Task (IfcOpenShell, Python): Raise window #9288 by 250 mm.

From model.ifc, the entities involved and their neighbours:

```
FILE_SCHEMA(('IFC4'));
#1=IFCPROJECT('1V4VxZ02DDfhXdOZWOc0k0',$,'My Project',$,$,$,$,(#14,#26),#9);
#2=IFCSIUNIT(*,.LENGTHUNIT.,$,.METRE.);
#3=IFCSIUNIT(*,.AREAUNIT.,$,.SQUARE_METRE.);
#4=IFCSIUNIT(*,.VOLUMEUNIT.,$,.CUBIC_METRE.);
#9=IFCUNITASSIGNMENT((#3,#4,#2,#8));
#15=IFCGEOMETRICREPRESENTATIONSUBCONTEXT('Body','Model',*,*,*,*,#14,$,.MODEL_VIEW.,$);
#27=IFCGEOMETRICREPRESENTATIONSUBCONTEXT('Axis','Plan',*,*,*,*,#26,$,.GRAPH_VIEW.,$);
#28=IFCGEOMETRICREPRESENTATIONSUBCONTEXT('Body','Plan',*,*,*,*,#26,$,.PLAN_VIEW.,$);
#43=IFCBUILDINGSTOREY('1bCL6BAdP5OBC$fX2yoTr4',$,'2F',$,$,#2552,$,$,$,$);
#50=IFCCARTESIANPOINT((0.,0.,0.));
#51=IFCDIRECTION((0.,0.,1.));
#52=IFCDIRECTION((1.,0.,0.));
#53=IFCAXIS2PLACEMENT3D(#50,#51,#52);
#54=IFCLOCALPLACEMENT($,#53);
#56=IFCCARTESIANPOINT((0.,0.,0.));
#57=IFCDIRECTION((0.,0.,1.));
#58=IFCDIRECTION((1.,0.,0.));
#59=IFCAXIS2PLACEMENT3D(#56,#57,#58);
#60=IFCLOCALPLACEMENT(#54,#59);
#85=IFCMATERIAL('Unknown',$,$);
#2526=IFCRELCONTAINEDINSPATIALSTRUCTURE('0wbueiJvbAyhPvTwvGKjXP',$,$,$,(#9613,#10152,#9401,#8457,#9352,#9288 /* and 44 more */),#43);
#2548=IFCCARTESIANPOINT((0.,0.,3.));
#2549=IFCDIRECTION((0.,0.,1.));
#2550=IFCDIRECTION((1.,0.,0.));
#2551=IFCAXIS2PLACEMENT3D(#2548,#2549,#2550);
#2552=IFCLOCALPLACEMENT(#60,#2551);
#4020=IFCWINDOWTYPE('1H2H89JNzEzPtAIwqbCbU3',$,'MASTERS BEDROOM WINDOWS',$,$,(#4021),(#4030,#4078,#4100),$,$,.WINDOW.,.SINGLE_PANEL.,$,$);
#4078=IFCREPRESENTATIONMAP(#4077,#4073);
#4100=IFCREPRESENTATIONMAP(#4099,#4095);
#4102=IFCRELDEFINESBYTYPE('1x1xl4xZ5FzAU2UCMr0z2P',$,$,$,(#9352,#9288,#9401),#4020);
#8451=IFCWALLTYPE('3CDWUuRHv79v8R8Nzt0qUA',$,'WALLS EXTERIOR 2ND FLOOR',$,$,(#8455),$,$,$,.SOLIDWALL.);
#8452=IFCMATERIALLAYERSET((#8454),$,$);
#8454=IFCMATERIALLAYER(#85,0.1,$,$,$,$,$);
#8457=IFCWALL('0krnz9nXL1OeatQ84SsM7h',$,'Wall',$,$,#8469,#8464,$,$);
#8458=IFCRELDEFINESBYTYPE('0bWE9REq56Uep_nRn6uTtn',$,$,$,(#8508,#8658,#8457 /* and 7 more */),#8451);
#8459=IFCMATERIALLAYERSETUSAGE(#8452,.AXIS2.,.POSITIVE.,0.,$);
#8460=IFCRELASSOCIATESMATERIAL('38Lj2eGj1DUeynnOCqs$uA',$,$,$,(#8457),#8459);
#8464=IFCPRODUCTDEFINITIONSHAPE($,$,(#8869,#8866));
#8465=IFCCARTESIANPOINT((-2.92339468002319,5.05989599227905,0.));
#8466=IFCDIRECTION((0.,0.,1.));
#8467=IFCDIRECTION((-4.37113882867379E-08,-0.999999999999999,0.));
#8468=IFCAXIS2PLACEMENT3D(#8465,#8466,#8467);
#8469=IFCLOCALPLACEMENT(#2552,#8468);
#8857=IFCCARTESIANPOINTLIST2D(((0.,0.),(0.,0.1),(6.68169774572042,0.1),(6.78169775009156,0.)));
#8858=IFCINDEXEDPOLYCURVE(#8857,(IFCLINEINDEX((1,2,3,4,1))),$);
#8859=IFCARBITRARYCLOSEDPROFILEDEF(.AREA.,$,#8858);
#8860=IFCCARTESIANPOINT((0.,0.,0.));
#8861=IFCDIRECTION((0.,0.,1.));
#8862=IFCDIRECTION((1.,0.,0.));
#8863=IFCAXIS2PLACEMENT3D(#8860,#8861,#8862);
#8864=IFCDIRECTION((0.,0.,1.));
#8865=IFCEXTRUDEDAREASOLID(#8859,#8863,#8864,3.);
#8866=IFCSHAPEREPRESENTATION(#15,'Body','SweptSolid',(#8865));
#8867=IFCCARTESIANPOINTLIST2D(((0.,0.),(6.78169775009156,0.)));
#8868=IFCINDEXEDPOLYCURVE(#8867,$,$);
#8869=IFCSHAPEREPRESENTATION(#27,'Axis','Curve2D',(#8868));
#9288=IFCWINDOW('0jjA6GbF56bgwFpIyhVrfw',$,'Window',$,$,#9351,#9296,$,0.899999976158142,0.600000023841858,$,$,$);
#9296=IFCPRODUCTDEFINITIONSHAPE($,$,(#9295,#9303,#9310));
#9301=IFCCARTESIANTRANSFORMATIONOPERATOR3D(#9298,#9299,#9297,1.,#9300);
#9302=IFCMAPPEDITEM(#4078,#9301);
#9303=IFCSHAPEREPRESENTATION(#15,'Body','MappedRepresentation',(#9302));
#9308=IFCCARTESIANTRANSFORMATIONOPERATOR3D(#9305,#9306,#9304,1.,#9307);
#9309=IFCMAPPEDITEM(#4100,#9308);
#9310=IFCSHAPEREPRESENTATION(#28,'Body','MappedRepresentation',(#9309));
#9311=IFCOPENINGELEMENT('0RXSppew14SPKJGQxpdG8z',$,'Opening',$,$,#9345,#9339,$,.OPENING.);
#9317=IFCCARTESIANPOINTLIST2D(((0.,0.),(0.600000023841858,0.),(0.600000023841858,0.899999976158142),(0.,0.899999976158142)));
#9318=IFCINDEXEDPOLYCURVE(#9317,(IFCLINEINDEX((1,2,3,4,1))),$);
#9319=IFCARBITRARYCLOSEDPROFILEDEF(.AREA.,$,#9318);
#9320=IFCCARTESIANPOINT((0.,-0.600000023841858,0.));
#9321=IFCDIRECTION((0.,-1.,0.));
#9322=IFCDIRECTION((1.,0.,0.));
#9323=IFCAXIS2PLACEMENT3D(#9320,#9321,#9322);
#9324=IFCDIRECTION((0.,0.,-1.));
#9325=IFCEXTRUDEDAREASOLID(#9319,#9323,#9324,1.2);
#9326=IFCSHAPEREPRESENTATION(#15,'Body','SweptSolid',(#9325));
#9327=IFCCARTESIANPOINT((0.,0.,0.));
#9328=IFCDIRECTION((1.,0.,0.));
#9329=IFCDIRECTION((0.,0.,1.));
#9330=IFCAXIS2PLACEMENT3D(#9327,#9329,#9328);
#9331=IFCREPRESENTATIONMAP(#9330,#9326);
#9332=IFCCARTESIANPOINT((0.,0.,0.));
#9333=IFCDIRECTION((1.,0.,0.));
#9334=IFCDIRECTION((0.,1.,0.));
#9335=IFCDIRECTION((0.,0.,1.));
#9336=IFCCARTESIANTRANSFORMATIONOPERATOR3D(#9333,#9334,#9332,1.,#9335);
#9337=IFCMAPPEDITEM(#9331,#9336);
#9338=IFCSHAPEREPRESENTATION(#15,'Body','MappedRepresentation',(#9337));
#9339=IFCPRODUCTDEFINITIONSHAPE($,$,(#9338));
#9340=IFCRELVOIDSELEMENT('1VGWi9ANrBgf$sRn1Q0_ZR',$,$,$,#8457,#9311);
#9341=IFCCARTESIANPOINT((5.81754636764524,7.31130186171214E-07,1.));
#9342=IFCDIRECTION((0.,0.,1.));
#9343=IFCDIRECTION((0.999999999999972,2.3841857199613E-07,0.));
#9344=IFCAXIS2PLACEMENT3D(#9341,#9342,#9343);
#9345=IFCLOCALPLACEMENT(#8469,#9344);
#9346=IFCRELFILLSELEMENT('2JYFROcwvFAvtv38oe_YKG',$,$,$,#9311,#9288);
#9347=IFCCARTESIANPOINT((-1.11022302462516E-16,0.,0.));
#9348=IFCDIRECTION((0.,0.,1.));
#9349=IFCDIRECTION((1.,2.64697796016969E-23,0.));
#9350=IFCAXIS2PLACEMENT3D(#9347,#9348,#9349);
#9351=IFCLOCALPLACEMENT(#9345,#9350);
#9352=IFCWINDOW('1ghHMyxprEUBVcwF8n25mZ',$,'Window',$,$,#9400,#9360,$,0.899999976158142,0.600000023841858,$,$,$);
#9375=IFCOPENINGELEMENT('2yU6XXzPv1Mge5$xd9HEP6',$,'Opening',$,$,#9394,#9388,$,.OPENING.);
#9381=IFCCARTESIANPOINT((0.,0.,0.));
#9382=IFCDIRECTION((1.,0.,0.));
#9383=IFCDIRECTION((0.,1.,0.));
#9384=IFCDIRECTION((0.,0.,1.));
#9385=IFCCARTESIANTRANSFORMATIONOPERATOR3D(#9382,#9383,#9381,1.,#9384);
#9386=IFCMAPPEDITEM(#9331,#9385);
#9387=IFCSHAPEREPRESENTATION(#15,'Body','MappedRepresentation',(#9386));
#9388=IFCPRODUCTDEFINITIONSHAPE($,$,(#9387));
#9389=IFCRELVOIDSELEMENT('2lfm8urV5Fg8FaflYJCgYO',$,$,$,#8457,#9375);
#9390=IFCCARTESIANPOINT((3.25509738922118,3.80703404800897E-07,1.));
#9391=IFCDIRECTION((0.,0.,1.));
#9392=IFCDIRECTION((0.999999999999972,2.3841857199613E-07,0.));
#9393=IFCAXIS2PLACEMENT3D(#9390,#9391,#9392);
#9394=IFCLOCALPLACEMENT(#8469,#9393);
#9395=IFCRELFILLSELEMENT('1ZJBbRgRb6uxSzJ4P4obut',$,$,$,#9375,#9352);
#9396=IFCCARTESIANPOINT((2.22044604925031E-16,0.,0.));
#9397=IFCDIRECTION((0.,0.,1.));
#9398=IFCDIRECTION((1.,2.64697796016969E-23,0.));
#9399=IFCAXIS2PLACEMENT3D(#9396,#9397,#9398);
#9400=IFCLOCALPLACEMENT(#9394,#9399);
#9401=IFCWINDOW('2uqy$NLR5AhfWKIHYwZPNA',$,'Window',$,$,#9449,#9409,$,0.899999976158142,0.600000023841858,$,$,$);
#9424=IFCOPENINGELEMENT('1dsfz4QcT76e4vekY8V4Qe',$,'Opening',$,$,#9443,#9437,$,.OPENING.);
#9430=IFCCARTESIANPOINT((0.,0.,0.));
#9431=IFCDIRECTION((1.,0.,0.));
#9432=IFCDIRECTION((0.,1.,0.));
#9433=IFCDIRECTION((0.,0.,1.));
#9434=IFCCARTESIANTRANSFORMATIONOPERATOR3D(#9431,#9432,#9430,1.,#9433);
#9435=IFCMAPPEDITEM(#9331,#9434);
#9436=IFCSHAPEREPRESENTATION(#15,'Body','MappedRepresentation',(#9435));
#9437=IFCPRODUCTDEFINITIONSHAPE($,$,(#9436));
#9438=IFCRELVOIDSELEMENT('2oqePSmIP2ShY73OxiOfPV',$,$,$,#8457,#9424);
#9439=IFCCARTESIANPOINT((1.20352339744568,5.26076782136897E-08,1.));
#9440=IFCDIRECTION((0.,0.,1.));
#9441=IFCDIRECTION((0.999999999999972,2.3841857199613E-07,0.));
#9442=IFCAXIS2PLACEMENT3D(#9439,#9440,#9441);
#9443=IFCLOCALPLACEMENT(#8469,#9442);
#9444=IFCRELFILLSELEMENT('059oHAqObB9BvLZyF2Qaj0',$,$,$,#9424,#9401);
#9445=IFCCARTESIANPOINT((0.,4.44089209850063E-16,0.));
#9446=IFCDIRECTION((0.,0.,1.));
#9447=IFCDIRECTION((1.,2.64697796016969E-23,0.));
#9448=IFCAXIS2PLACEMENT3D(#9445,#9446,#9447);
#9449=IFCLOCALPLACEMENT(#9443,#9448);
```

```python
import numpy as np
import ifcopenshell
import ifcopenshell.api.geometry
import ifcopenshell.util.placement
import ifcopenshell.util.unit

model = ifcopenshell.open("model.ifc")
unit_scale = ifcopenshell.util.unit.calculate_unit_scale(model)

window = model.by_id(9288)
opening = window.FillsVoids[0].RelatingOpeningElement
dz = 0.25

shift = np.array([0.0, 0.0, dz])
# The window is placed relative to its opening, so it follows when the opening moves.
matrix = ifcopenshell.util.placement.get_local_placement(opening.ObjectPlacement)
matrix[:3, 3] += shift
ifcopenshell.api.geometry.edit_object_placement(
    model, product=opening, matrix=matrix, is_si=False, should_transform_children=True
)

print(f"moved by {dz * unit_scale:+.3f} m")

model.write("model_edited.ifc")
```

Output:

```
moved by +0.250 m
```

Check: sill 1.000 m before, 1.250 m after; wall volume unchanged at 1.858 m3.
